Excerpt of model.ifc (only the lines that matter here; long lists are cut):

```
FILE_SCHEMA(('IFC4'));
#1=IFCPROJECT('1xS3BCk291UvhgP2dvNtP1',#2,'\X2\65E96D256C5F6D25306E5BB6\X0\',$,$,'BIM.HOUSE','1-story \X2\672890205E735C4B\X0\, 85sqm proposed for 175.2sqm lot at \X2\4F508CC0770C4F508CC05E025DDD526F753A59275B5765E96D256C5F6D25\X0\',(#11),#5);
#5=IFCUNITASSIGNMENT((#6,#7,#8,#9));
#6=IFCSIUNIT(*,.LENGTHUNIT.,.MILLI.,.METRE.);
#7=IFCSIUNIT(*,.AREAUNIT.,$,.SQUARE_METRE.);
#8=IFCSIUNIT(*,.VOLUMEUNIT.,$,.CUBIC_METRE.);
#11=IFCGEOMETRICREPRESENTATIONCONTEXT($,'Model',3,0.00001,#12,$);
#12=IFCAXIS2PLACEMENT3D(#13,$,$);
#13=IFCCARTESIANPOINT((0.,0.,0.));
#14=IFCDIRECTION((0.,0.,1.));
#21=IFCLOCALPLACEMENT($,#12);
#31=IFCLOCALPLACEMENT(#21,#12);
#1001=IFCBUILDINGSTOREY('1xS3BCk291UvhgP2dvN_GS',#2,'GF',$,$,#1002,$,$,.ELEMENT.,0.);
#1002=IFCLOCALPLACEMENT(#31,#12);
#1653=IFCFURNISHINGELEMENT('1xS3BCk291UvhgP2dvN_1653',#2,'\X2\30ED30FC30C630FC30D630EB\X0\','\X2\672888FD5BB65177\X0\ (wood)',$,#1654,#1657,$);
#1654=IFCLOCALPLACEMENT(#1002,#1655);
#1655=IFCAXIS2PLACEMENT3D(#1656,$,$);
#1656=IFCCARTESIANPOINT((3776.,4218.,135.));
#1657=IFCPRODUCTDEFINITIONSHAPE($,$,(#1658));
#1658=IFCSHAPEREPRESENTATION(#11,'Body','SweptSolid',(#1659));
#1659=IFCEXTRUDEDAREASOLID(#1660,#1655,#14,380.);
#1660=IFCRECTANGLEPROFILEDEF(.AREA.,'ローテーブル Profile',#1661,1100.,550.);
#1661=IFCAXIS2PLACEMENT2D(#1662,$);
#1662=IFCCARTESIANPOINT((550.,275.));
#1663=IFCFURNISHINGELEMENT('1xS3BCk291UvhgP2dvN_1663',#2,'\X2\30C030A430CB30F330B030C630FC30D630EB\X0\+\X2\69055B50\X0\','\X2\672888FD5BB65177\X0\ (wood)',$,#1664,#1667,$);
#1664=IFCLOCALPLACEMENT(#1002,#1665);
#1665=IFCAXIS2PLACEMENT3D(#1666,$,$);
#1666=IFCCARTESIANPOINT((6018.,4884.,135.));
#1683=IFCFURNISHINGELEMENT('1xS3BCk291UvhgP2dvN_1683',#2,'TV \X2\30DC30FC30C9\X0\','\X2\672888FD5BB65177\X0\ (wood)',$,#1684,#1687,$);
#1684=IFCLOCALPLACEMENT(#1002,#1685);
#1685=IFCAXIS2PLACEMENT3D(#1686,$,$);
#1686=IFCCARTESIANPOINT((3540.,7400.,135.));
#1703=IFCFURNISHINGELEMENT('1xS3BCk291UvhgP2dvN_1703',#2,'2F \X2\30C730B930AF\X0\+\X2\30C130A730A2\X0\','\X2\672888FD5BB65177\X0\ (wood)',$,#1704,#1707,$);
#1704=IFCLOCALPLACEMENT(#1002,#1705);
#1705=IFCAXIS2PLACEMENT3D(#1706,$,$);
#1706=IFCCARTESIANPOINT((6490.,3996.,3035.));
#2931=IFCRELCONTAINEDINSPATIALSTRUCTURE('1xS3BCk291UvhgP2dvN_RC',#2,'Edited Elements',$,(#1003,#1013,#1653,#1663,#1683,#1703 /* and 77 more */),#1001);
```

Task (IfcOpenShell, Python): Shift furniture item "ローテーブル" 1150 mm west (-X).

```python
import ifcopenshell
import ifcopenshell.api.geometry
import ifcopenshell.util.placement

model = ifcopenshell.open("model.ifc")

item = model.by_id(1653)
matrix = ifcopenshell.util.placement.get_local_placement(item.ObjectPlacement)
matrix[0, 3] -= 1150.0
ifcopenshell.api.geometry.edit_object_placement(model, product=item, matrix=matrix, is_si=False)

print(ifcopenshell.util.placement.get_local_placement(item.ObjectPlacement).round(3) + 0.0)

model.write("model_v2.ifc")
```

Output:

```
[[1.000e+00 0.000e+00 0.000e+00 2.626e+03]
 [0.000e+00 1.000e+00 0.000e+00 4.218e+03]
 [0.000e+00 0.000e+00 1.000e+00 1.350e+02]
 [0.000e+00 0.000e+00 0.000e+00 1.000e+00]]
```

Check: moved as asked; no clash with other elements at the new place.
